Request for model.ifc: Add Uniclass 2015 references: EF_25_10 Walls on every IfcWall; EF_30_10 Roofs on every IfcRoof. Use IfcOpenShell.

First a look at what the model holds.

```python
import ifcopenshell

model = ifcopenshell.open("model.ifc")
print(model.schema)
print("classifications:", [c.Name for c in model.by_type("IfcClassification")])
for ifc_class in ("IfcDoor", "IfcRoof", "IfcStair", "IfcWall", "IfcWindow"):
    print(ifc_class, len(model.by_type(ifc_class)))
```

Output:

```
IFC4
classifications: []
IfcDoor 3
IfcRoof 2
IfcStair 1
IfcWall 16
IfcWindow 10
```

```python
import ifcopenshell
import ifcopenshell.api.classification

model = ifcopenshell.open("model.ifc")

system = ifcopenshell.api.classification.add_classification(model, classification="Uniclass 2015")

codes = {
    "IfcWall": ("EF_25_10", "Walls"),
    "IfcRoof": ("EF_30_10", "Roofs"),
}
for ifc_class, (code, name) in codes.items():
    products = model.by_type(ifc_class)
    ifcopenshell.api.classification.add_reference(
        model, products=products, classification=system, identification=code, name=name
    )
    print(code, len(products))

model.write("model_rev.ifc")
```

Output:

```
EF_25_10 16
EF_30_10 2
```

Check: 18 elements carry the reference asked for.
